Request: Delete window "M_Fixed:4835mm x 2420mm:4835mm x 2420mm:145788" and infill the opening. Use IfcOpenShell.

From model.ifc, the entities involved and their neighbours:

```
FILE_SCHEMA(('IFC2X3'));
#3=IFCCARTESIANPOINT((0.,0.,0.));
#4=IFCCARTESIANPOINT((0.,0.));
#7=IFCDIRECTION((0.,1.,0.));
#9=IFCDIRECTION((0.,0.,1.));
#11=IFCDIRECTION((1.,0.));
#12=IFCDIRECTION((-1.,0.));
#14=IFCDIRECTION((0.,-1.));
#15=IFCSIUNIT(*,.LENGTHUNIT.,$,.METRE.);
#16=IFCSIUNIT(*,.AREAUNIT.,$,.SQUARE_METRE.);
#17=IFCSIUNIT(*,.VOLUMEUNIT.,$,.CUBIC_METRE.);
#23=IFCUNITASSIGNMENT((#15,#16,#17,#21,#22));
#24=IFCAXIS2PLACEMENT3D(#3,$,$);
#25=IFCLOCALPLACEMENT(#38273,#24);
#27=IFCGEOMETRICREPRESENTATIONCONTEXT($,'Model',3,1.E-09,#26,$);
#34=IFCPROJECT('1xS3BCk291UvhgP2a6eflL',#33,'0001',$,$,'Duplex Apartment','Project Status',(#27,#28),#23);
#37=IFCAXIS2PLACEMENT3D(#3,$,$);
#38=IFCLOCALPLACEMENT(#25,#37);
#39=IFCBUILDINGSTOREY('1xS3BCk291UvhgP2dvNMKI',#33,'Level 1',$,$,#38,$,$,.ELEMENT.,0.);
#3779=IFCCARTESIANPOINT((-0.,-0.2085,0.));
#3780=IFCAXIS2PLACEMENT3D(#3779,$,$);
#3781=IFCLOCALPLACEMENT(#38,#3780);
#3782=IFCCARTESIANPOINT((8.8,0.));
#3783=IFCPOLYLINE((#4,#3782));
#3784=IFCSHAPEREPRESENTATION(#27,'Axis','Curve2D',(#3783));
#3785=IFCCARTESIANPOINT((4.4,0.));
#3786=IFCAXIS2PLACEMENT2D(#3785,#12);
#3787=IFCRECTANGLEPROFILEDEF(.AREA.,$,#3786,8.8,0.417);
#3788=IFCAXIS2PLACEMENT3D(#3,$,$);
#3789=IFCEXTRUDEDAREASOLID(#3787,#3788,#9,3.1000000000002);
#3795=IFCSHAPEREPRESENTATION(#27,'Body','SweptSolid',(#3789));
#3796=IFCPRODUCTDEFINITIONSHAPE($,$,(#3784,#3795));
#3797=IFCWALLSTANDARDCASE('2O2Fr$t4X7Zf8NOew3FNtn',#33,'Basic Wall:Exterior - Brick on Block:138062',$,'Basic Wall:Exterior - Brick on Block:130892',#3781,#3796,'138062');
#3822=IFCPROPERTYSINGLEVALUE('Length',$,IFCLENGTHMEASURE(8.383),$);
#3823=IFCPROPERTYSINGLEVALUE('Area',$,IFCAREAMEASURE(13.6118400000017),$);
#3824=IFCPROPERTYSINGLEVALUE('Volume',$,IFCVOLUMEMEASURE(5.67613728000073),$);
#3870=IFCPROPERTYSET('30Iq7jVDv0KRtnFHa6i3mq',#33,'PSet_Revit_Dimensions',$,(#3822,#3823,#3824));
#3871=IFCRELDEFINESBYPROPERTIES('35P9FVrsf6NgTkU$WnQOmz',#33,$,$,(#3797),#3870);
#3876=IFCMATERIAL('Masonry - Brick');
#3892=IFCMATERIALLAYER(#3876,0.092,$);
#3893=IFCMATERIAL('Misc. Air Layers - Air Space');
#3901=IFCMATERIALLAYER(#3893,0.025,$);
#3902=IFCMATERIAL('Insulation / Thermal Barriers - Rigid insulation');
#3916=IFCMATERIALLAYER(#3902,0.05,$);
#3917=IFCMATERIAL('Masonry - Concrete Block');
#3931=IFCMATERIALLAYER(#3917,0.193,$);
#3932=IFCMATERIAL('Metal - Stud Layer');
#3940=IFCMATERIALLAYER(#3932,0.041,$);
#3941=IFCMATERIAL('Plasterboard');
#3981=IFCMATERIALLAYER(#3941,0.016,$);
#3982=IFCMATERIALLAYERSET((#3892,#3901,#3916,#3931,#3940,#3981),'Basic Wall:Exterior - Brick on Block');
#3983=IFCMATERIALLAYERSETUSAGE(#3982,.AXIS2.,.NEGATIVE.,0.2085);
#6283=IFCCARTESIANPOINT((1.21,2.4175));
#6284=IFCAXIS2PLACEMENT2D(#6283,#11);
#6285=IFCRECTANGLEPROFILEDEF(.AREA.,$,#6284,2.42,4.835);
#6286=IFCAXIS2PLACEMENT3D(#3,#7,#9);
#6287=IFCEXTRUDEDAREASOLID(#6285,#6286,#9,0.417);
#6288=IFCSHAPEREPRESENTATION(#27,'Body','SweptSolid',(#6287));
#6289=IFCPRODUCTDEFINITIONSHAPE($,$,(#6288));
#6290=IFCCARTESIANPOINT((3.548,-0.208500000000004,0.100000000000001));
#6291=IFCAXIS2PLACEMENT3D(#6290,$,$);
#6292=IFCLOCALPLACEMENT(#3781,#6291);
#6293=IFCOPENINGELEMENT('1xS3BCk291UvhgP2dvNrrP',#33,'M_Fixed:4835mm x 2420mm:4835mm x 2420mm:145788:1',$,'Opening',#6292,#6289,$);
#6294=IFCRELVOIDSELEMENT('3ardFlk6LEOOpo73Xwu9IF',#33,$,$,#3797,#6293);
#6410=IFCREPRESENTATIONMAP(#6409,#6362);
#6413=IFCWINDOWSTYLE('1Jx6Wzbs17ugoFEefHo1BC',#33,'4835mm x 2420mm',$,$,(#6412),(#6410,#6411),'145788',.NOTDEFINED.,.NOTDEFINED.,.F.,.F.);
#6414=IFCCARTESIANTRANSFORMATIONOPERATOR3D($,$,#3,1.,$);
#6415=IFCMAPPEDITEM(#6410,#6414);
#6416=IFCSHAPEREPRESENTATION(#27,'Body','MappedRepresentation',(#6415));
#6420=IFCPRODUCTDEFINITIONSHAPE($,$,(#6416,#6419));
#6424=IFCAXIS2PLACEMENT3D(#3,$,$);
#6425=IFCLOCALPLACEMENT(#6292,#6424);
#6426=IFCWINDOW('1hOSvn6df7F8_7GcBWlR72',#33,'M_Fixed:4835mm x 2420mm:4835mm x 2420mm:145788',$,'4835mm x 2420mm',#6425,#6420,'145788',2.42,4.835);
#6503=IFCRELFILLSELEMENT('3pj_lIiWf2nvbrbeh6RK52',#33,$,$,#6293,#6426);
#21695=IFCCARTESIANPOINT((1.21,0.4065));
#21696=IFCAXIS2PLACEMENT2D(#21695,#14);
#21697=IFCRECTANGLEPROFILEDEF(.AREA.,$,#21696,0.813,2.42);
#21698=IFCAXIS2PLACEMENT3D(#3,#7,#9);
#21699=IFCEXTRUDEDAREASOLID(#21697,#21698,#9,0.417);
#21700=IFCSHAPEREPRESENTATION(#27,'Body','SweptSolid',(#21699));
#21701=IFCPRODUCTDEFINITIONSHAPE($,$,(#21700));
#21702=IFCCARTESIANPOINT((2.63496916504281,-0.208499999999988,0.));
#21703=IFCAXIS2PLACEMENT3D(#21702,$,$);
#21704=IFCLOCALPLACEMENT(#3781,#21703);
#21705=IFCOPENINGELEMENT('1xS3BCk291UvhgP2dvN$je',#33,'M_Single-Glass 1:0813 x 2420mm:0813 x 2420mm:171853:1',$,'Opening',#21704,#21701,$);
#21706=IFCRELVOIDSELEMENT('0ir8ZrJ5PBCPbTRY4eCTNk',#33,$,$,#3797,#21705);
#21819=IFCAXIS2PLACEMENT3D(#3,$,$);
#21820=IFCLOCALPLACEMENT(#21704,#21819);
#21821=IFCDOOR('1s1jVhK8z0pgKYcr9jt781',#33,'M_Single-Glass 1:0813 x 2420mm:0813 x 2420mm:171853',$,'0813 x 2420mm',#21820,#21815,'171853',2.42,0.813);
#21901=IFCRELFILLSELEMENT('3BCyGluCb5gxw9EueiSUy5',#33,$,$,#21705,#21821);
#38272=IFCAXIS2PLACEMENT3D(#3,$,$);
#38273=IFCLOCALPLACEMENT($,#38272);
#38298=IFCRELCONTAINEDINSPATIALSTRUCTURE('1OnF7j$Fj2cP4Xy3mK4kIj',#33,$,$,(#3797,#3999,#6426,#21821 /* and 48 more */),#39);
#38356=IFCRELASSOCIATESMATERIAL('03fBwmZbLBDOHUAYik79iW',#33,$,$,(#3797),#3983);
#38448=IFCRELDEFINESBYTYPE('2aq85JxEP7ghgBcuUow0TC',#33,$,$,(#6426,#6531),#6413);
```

```python
import ifcopenshell
import ifcopenshell.api.feature
import ifcopenshell.api.pset
import ifcopenshell.api.root
import ifcopenshell.geom
import ifcopenshell.util.element
import ifcopenshell.util.shape
import ifcopenshell.util.unit

model = ifcopenshell.open("model.ifc")
area_scale = ifcopenshell.util.unit.calculate_unit_scale(model, "AREAUNIT")
volume_scale = ifcopenshell.util.unit.calculate_unit_scale(model, "VOLUMEUNIT")
settings = ifcopenshell.geom.settings()


def volume(element):
    """Net volume in cubic metres, openings subtracted."""
    shape = ifcopenshell.geom.create_shape(settings, element)
    return ifcopenshell.util.shape.get_volume(shape.geometry)


window = model.by_guid("1hOSvn6df7F8_7GcBWlR72")
opening = window.FillsVoids[0].RelatingOpeningElement
wall = opening.VoidsElements[0].RelatingBuildingElement
before = volume(wall)

ifcopenshell.api.root.remove_product(model, product=window)
ifcopenshell.api.feature.remove_feature(model, feature=opening)

after = volume(wall)
thickness = 0.417  # wall thickness in metres

# Update the wall's stored quantities.
pset = model.by_id(ifcopenshell.util.element.get_pset(wall, "PSet_Revit_Dimensions", should_inherit=False)["id"])
ifcopenshell.api.pset.edit_pset(model, pset=pset, properties={
    "Area": model.create_entity("IfcAreaMeasure", after / thickness / area_scale),
    "Volume": model.create_entity("IfcVolumeMeasure", after / volume_scale),
})

print(f"wall volume {before:.3f} -> {after:.3f} m3")

model.write("model_updated.ifc")
```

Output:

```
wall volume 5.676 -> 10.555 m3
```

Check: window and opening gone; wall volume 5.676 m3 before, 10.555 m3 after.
